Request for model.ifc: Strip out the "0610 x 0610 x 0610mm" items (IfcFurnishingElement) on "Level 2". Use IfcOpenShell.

First a look at what the model holds.

```python
import ifcopenshell
import ifcopenshell.util.element

model = ifcopenshell.open("model.ifc")
print(model.schema)
storey = next(s for s in model.by_type("IfcBuildingStorey") if s.Name == "Level 2")
furniture = [e for e in ifcopenshell.util.element.get_decomposition(storey) if e.is_a("IfcFurnishingElement")]
seen = {}
for e in furniture:
    element_type = ifcopenshell.util.element.get_type(e)
    name = element_type.Name if element_type not in (None, e) else None
    seen[name] = seen.get(name, 0) + 1
for name, count in sorted(seen.items(), key=str):
    print(count, "x", name)
```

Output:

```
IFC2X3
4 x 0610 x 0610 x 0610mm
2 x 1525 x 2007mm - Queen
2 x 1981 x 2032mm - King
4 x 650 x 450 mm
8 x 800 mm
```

```python
import ifcopenshell
import ifcopenshell.api.root
import ifcopenshell.util.element

model = ifcopenshell.open("model.ifc")

storey = next(s for s in model.by_type("IfcBuildingStorey") if s.Name == "Level 2")
furniture = [e for e in ifcopenshell.util.element.get_decomposition(storey) if e.is_a("IfcFurnishingElement")]
targets = [e for e in furniture if (t := ifcopenshell.util.element.get_type(e)) not in (None, e) and t.Name == "0610 x 0610 x 0610mm"]

for e in targets:
    ifcopenshell.api.root.remove_product(model, product=e)
print(len(targets), "removed")

model.write("model_v2.ifc")
```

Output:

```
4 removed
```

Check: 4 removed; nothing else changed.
